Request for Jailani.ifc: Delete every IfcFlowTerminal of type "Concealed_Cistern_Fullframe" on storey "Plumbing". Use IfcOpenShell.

First a look at what the model holds.

```python
import ifcopenshell
import ifcopenshell.util.element

model = ifcopenshell.open("Jailani.ifc")
print(model.schema)
storey = next(s for s in model.by_type("IfcBuildingStorey") if s.Name == "Plumbing")
terminals = [e for e in ifcopenshell.util.element.get_decomposition(storey) if e.is_a("IfcFlowTerminal")]
seen = {}
for e in terminals:
    element_type = ifcopenshell.util.element.get_type(e)
    name = element_type.Name if element_type not in (None, e) else None
    seen[name] = seen.get(name, 0) + 1
for name, count in sorted(seen.items(), key=str):
    print(count, "x", name)
```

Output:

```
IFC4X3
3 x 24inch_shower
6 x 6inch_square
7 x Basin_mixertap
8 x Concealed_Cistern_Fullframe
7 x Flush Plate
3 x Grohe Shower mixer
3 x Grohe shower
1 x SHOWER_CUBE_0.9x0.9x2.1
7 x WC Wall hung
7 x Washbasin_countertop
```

```python
import ifcopenshell
import ifcopenshell.api.root
import ifcopenshell.util.element

model = ifcopenshell.open("Jailani.ifc")

storey = next(s for s in model.by_type("IfcBuildingStorey") if s.Name == "Plumbing")
terminals = [e for e in ifcopenshell.util.element.get_decomposition(storey) if e.is_a("IfcFlowTerminal")]
targets = [e for e in terminals if (t := ifcopenshell.util.element.get_type(e)) not in (None, e) and t.Name == "Concealed_Cistern_Fullframe"]

for e in targets:
    ifcopenshell.api.root.remove_product(model, product=e)
print(len(targets), "removed")

model.write("Jailani_updated.ifc")
```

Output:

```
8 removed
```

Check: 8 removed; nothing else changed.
